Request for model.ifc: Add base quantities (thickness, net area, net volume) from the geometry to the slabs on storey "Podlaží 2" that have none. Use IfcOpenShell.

First a look at what the model holds.

```python
import ifcopenshell
import ifcopenshell.util.element
import ifcopenshell.util.unit

model = ifcopenshell.open("model.ifc")
print(model.schema)
for unit_type in ("LENGTHUNIT", "AREAUNIT", "VOLUMEUNIT"):
    print(unit_type, ifcopenshell.util.unit.calculate_unit_scale(model, unit_type))
storey = next(s for s in model.by_type("IfcBuildingStorey") if s.Name == "Podlaží 2")
slabs = [e for e in ifcopenshell.util.element.get_decomposition(storey) if e.is_a("IfcSlab")]
for e in sorted(slabs, key=lambda e: e.id()):
    print(e.id(), e.is_a(), e.Name, list(ifcopenshell.util.element.get_psets(e, qtos_only=True)), sep=" | ")
```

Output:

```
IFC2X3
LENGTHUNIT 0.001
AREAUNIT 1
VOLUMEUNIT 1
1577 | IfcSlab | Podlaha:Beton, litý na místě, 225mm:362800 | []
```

```python
import ifcopenshell
import ifcopenshell.api.pset
import ifcopenshell.geom
import ifcopenshell.util.element
import ifcopenshell.util.shape
import ifcopenshell.util.unit

model = ifcopenshell.open("model.ifc")
unit_scale = ifcopenshell.util.unit.calculate_unit_scale(model)
area_scale = ifcopenshell.util.unit.calculate_unit_scale(model, "AREAUNIT")
volume_scale = ifcopenshell.util.unit.calculate_unit_scale(model, "VOLUMEUNIT")
settings = ifcopenshell.geom.settings()

storey = next(s for s in model.by_type("IfcBuildingStorey") if s.Name == "Podlaží 2")
slabs = [e for e in ifcopenshell.util.element.get_decomposition(storey) if e.is_a("IfcSlab")]

for e in sorted(slabs, key=lambda e: e.id()):
    if ifcopenshell.util.element.get_psets(e, qtos_only=True, should_inherit=False):
        continue
    # Geometry comes back in metres, in the element's own axes.
    shape = ifcopenshell.geom.create_shape(settings, e)
    values = {
        "Width": ifcopenshell.util.shape.get_z(shape.geometry) / unit_scale,
        "NetArea": ifcopenshell.util.shape.get_footprint_area(shape.geometry) / area_scale,
        "NetVolume": ifcopenshell.util.shape.get_volume(shape.geometry) / volume_scale,
    }
    qto = ifcopenshell.api.pset.add_qto(model, product=e, name="BaseQuantities")
    ifcopenshell.api.pset.edit_qto(model, qto=qto, properties=values)
    print(e.id(), {k: round(v, 3) for k, v in values.items()})

model.write("model-out.ifc")
```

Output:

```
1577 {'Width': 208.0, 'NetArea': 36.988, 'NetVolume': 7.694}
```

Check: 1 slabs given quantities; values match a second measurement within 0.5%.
